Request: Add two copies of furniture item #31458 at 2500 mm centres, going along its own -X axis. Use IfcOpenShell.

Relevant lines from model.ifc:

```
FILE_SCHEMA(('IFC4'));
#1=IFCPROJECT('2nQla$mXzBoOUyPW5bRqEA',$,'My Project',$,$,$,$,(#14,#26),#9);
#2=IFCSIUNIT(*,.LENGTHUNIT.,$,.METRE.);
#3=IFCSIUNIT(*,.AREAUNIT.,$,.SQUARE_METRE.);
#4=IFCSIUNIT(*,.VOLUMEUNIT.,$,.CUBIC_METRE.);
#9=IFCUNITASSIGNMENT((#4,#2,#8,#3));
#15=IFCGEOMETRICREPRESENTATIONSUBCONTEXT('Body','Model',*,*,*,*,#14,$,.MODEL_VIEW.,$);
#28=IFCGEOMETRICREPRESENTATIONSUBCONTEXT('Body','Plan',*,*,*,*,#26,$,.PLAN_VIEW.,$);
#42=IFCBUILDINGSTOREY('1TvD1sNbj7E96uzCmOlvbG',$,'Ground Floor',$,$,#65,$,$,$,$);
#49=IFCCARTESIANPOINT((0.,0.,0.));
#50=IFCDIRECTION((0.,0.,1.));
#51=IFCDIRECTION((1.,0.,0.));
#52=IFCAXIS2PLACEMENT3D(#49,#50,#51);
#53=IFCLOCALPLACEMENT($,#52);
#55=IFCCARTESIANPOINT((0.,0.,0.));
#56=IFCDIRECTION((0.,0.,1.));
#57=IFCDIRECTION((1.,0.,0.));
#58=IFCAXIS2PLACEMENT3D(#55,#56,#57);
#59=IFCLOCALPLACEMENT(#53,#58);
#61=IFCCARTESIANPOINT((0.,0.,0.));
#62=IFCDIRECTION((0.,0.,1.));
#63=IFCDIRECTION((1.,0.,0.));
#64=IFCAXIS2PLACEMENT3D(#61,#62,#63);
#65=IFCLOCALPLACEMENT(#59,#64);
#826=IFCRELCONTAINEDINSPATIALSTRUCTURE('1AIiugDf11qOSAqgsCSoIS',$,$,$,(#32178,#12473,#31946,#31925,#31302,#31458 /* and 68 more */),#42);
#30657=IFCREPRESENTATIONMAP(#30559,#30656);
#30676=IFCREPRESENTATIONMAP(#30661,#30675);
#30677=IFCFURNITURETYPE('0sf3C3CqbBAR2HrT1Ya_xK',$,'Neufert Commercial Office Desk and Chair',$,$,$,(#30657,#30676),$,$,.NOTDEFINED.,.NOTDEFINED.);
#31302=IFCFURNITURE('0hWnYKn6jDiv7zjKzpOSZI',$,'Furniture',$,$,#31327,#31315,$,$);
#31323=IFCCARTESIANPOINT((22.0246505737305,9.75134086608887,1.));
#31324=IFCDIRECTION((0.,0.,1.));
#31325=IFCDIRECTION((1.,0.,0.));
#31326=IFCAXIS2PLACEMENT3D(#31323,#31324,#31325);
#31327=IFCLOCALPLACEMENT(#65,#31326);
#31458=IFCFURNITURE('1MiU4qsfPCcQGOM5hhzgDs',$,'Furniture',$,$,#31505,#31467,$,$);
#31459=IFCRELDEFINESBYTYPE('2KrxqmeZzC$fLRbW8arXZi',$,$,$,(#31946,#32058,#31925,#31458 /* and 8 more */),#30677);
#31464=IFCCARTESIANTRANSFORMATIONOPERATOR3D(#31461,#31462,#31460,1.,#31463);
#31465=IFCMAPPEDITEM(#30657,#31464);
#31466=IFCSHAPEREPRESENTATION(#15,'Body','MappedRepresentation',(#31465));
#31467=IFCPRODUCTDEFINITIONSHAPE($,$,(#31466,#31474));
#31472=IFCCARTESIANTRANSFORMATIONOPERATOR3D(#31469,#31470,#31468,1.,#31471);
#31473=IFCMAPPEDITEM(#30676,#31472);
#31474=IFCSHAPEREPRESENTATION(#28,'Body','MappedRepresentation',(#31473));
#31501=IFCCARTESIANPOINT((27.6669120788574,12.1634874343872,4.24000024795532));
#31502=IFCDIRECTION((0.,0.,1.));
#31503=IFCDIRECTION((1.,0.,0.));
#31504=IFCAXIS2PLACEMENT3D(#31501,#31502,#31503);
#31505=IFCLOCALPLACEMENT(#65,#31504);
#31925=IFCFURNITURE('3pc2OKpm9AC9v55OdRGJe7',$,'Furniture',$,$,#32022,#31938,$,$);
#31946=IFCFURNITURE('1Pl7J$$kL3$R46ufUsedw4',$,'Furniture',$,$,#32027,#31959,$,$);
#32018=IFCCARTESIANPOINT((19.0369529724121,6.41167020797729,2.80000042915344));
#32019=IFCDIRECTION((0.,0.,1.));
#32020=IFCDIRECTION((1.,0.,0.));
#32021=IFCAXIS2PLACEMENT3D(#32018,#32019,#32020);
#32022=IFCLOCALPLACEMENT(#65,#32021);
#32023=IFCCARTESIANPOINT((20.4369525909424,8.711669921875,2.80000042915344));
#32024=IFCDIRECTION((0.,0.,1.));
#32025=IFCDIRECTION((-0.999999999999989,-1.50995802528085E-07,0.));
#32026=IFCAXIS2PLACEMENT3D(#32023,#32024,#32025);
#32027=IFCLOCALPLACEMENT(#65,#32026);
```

```python
import ifcopenshell
import ifcopenshell.api.geometry
import ifcopenshell.api.root
import ifcopenshell.util.element
import ifcopenshell.util.placement

model = ifcopenshell.open("model.ifc")

source = model.by_guid("1MiU4qsfPCcQGOM5hhzgDs")
base = ifcopenshell.util.placement.get_local_placement(source.ObjectPlacement)
step = -base[:3, 0] * 2.5

for i in range(1, 3):
    copy = ifcopenshell.api.root.copy_class(model, product=source)
    copy.Representation = ifcopenshell.util.element.copy_deep(
        model, source.Representation, exclude=["IfcGeometricRepresentationContext", "IfcRepresentationMap"]
    )
    matrix = base.copy()
    matrix[:3, 3] += i * step
    print("added at", matrix[:3, 3].round(3) + 0.0)
    ifcopenshell.api.geometry.edit_object_placement(model, product=copy, matrix=matrix, is_si=False)

model.write("model_updated.ifc")
```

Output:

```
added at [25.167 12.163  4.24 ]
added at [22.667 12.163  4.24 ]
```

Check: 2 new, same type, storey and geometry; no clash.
